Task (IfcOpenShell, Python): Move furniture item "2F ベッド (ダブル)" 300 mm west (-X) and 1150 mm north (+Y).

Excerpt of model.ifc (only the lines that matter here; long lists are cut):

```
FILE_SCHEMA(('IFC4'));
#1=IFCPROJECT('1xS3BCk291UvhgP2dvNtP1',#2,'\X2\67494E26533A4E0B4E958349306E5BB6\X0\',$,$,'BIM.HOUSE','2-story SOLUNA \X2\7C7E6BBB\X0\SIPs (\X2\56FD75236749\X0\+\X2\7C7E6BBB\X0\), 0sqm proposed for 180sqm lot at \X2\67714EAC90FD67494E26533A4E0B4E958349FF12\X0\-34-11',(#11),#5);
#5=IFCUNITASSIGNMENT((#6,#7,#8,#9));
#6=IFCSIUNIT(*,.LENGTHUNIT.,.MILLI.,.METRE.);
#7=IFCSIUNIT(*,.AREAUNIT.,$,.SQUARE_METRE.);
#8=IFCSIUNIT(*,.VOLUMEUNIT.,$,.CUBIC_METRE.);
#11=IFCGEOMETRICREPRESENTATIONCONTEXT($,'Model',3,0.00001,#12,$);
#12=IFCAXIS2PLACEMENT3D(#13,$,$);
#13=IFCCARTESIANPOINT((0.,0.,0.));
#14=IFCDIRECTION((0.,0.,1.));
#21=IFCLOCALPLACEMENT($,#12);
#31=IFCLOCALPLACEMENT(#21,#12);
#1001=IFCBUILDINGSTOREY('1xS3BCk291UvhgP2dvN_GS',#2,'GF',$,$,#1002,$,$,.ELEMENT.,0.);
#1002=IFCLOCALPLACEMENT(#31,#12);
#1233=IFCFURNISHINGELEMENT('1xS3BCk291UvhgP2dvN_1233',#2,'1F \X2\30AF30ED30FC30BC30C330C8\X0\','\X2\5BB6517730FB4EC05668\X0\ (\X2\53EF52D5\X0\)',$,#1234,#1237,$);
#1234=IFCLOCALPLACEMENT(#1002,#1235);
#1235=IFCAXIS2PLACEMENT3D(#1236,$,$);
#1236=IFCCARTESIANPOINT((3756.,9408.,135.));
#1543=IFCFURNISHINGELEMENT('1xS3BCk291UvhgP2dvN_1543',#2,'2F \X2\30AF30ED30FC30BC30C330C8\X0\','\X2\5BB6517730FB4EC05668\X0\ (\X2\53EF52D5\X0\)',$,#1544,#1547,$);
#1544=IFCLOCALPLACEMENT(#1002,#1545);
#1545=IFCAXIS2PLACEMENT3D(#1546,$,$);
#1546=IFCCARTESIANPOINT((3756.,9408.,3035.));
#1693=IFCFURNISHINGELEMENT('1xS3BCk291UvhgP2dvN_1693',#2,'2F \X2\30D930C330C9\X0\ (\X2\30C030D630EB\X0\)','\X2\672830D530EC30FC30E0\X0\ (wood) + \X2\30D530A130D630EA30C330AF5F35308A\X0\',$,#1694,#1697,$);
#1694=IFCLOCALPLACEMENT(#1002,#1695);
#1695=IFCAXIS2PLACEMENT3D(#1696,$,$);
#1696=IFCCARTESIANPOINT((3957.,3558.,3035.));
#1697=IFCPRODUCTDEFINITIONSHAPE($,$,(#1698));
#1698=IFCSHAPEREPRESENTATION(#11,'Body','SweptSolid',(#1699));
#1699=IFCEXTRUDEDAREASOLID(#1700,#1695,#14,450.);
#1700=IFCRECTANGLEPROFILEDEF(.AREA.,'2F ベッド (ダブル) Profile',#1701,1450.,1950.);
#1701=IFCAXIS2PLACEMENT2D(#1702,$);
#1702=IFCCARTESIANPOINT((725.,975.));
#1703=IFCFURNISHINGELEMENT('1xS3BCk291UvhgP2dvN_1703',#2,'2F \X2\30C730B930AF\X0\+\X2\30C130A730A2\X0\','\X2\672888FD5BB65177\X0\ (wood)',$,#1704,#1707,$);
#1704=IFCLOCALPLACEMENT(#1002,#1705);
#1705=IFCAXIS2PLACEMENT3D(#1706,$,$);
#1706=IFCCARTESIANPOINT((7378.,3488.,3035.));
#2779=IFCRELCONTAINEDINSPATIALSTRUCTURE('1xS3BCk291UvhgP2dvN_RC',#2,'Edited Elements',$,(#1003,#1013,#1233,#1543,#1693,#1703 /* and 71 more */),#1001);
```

```python
import ifcopenshell
import ifcopenshell.api.geometry
import ifcopenshell.util.placement
import ifcopenshell.util.unit

model = ifcopenshell.open("model.ifc")
unit_scale = ifcopenshell.util.unit.calculate_unit_scale(model)

item = model.by_guid("1xS3BCk291UvhgP2dvN_1693")
matrix = ifcopenshell.util.placement.get_local_placement(item.ObjectPlacement)
matrix[0, 3] -= 0.3 / unit_scale
matrix[1, 3] += 1.15 / unit_scale
ifcopenshell.api.geometry.edit_object_placement(model, product=item, matrix=matrix, is_si=False)

print(ifcopenshell.util.placement.get_local_placement(item.ObjectPlacement).round(3) + 0.0)

model.write("model_rev.ifc")
```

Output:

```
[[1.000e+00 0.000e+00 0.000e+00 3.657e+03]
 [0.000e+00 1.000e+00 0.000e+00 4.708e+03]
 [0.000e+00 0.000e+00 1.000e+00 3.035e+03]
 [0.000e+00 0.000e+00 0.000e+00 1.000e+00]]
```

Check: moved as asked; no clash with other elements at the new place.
